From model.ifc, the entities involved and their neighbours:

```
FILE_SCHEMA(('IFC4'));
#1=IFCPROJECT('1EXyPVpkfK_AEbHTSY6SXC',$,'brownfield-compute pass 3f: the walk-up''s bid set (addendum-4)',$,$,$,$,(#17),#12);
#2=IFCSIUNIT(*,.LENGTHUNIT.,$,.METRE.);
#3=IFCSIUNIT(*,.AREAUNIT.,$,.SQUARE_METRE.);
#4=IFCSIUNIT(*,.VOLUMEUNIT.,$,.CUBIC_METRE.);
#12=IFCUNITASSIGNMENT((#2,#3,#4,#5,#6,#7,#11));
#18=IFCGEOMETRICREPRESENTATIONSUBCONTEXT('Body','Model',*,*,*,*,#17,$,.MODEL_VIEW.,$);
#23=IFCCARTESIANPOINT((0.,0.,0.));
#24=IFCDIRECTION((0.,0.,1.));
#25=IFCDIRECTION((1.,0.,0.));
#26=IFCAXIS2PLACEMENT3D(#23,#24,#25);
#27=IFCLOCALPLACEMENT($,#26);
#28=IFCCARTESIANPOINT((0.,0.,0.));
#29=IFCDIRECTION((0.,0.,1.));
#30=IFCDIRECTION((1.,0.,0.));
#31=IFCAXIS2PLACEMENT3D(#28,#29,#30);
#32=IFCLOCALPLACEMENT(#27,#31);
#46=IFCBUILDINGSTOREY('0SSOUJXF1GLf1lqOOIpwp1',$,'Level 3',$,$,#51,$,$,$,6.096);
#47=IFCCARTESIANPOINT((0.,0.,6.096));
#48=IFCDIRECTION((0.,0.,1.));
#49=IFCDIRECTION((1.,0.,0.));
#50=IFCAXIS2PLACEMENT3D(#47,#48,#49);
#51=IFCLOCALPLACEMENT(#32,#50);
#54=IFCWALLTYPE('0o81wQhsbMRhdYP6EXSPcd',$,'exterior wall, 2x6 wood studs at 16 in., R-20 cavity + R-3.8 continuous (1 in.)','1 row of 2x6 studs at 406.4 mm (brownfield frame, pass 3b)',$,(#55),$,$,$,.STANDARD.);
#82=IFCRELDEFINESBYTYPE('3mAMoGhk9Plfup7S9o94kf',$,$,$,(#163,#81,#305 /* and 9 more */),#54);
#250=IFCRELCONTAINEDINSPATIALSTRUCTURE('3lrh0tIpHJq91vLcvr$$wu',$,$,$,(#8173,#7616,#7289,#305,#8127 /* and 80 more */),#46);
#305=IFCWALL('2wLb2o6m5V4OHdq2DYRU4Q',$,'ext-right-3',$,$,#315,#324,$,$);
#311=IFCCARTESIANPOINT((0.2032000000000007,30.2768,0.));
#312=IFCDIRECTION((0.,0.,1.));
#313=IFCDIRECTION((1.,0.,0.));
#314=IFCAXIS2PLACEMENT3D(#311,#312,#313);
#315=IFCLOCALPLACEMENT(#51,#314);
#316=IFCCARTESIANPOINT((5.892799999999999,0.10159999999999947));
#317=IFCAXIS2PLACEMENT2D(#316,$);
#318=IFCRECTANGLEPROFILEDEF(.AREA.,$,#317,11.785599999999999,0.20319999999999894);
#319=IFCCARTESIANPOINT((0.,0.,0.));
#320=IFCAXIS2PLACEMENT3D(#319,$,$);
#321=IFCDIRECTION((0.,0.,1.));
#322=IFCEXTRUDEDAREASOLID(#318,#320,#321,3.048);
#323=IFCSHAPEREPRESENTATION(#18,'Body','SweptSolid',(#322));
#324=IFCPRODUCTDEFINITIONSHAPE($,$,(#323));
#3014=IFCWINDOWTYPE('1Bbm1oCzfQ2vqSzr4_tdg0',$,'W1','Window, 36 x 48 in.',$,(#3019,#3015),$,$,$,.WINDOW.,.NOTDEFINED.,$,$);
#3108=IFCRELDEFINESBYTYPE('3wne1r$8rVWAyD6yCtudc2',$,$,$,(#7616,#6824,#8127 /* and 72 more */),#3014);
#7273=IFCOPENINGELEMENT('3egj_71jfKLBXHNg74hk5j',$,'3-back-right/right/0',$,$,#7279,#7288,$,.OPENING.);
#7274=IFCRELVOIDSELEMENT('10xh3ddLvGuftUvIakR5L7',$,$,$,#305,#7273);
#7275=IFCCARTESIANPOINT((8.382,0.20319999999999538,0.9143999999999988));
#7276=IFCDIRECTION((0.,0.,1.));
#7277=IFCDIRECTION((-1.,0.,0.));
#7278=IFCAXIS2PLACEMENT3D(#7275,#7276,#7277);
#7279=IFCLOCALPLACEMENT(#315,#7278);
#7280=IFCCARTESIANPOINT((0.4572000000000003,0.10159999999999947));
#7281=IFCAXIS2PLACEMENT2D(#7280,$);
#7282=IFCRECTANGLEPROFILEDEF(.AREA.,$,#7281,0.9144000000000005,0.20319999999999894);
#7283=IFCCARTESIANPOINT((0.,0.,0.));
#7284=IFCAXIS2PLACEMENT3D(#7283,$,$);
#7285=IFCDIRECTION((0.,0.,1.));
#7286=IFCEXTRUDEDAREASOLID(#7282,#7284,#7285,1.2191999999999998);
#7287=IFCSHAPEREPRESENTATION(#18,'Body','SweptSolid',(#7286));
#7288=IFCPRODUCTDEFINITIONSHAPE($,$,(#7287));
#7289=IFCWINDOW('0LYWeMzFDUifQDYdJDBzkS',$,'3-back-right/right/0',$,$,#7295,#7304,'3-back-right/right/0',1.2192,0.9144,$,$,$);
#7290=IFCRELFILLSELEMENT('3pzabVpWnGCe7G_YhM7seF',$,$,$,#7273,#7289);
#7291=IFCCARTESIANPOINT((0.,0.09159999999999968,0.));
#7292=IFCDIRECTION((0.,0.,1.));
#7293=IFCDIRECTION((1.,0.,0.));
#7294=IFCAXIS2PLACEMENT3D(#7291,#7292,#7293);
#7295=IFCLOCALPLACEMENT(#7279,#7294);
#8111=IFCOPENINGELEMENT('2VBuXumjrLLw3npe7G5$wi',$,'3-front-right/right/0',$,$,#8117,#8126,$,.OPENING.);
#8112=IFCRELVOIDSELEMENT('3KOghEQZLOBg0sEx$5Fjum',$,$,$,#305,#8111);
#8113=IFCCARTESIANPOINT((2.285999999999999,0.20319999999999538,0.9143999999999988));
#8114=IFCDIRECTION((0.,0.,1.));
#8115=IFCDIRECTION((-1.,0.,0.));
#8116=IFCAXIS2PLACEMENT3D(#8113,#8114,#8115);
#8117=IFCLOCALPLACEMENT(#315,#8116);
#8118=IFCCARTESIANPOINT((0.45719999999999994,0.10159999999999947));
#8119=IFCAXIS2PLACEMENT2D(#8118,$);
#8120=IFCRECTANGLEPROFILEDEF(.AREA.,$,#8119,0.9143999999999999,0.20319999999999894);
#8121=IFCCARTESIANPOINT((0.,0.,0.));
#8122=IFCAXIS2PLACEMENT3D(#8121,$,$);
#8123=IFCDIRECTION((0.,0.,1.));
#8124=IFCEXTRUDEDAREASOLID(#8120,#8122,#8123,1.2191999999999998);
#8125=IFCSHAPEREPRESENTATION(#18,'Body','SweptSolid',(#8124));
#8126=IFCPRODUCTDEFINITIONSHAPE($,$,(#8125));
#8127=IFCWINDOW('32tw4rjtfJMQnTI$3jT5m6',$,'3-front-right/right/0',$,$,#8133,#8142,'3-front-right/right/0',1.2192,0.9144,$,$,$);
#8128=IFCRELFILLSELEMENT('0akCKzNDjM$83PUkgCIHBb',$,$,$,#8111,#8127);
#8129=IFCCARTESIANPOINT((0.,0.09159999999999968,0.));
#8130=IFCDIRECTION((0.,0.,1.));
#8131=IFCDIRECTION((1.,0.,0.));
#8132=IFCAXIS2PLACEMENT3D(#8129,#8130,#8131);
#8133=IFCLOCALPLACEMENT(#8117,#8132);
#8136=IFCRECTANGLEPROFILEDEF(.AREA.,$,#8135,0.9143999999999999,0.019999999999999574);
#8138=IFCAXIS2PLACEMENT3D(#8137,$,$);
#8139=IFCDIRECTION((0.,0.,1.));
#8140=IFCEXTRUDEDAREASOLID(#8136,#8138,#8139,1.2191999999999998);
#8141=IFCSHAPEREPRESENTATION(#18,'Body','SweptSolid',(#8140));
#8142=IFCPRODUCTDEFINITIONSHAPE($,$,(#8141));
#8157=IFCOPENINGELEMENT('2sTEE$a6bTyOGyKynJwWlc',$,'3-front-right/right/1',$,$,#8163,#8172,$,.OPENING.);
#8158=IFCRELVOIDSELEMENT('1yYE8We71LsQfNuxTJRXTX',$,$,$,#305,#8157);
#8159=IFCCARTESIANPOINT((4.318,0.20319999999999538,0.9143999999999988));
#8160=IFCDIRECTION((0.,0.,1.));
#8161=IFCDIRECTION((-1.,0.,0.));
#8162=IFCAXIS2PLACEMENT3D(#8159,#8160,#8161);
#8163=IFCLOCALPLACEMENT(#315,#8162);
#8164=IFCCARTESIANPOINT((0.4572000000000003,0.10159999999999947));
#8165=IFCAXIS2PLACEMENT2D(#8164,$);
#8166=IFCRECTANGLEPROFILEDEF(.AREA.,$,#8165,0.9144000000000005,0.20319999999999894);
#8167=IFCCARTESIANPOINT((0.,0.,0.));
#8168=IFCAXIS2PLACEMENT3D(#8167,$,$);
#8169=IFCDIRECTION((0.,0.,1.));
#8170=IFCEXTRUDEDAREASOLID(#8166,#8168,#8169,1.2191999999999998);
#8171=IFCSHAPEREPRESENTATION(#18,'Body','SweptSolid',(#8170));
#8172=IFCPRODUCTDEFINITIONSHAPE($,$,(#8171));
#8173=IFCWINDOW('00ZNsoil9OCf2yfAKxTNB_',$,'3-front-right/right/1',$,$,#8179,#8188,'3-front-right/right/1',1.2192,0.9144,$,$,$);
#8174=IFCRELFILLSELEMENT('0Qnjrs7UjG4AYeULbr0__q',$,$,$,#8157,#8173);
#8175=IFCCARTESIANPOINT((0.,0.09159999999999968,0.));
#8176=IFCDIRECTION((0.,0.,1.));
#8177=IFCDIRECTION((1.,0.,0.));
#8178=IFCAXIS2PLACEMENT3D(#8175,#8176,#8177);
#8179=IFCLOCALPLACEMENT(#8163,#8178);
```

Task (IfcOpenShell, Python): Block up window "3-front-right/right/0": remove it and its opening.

```python
import ifcopenshell
import ifcopenshell.api.feature
import ifcopenshell.api.root
import ifcopenshell.geom
import ifcopenshell.util.shape

model = ifcopenshell.open("model.ifc")
settings = ifcopenshell.geom.settings()


def volume(element):
    """Net volume in cubic metres, openings subtracted."""
    shape = ifcopenshell.geom.create_shape(settings, element)
    return ifcopenshell.util.shape.get_volume(shape.geometry)


window = model.by_id(8127)
opening = window.FillsVoids[0].RelatingOpeningElement
wall = opening.VoidsElements[0].RelatingBuildingElement
before = volume(wall)

ifcopenshell.api.root.remove_product(model, product=window)
ifcopenshell.api.feature.remove_feature(model, feature=opening)

after = volume(wall)

print(f"wall volume {before:.3f} -> {after:.3f} m3")

model.write("model_v2.ifc")
```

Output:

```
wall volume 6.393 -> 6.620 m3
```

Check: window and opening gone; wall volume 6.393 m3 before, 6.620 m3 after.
